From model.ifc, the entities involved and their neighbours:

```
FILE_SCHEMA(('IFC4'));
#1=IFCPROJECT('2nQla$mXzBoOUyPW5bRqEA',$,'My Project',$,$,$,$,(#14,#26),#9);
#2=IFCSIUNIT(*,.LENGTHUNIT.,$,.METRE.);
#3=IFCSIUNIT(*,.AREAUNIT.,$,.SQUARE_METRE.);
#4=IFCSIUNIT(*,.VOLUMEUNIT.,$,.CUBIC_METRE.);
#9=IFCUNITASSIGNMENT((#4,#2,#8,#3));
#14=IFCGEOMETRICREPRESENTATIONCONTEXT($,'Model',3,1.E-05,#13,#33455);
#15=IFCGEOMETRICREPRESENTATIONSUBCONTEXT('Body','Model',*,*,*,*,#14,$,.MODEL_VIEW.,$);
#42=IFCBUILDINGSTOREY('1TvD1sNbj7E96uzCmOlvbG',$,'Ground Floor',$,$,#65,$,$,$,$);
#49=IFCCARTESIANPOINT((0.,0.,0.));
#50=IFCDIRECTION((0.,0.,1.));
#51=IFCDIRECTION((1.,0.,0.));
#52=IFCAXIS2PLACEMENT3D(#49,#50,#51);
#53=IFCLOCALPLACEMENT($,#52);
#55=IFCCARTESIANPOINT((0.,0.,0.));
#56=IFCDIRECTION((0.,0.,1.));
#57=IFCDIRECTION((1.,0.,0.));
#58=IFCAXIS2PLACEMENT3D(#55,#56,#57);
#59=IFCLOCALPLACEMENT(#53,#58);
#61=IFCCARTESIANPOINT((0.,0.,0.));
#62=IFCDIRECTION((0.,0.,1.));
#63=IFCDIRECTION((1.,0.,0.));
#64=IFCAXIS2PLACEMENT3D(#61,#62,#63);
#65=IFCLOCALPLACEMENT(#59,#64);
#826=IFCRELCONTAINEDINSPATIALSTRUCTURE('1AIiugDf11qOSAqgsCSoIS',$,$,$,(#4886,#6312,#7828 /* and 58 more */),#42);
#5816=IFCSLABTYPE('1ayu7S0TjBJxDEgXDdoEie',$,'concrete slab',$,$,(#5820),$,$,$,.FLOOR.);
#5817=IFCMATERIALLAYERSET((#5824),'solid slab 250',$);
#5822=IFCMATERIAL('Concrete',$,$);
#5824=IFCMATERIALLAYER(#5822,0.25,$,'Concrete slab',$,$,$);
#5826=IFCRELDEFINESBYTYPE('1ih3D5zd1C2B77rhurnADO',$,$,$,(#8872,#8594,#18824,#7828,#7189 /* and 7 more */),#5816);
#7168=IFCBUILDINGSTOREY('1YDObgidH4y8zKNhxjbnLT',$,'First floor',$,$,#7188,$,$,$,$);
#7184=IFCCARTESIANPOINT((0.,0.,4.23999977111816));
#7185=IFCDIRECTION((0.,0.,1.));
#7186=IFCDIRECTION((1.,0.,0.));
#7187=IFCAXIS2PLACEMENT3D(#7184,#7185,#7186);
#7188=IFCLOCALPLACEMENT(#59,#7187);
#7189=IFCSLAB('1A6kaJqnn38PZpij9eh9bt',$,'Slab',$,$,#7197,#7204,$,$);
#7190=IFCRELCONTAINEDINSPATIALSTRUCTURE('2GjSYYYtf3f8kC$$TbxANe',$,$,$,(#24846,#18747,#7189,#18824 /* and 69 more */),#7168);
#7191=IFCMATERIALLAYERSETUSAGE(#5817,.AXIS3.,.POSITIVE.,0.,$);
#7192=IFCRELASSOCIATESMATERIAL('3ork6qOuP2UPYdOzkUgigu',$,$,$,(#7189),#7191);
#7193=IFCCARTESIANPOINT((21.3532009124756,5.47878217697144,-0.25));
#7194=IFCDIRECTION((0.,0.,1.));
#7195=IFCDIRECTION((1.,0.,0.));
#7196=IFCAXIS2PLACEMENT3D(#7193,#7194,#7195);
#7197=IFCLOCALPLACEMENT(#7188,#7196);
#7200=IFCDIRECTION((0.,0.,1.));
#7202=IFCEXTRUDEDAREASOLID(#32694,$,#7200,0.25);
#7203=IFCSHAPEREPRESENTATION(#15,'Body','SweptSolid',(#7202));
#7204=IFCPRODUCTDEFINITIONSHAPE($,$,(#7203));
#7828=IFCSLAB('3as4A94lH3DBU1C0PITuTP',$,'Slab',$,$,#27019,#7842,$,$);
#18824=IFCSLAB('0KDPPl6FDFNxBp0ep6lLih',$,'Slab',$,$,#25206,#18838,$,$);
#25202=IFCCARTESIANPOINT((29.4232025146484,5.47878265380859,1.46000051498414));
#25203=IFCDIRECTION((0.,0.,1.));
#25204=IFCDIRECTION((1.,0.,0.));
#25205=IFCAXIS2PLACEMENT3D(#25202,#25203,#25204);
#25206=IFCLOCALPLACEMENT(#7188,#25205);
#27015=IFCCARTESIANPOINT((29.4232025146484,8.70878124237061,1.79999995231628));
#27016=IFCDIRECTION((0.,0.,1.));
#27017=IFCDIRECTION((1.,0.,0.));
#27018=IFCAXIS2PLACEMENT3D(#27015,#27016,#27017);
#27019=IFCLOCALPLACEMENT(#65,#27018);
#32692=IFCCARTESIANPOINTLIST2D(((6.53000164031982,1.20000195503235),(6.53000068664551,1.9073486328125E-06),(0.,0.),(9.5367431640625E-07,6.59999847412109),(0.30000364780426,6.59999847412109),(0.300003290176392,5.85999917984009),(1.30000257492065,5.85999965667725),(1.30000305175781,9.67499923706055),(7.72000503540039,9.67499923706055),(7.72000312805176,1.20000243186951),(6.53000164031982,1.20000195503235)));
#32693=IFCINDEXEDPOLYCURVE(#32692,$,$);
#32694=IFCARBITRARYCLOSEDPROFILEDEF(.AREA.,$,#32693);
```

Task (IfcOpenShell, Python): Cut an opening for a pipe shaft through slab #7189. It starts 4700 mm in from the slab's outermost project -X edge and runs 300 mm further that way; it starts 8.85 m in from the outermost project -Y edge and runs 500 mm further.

```python
import numpy as np
import ifcopenshell
import ifcopenshell.api.feature
import ifcopenshell.api.geometry
import ifcopenshell.api.root
import ifcopenshell.geom
import ifcopenshell.util.placement
import ifcopenshell.util.representation
import ifcopenshell.util.shape
import ifcopenshell.util.unit

model = ifcopenshell.open("model.ifc")
unit_scale = ifcopenshell.util.unit.calculate_unit_scale(model)
settings = ifcopenshell.geom.settings()


def volume(element):
    """Net volume in cubic metres, openings subtracted."""
    shape = ifcopenshell.geom.create_shape(settings, element)
    return ifcopenshell.util.shape.get_volume(shape.geometry)


slab = model.by_id(7189)
before = volume(slab)

# Extent in the slab's own axes, in metres. The edges named are its -X and -Y sides.
slab_shape = ifcopenshell.geom.create_shape(settings, slab)
vertices = ifcopenshell.util.shape.get_vertices(slab_shape.geometry)
x_min, y_min, bottom = vertices.min(axis=0)
top = vertices[:, 2].max()

opening = ifcopenshell.api.root.create_entity(model, ifc_class="IfcOpeningElement", name="Pipe shaft opening", predefined_type="OPENING")
context = ifcopenshell.util.representation.get_context(model, "Model", "Body", "MODEL_VIEW")
width, depth = 0.3, 0.5
outline = [(0.0, 0.0), (width, 0.0), (width, depth), (0.0, depth), (0.0, 0.0)]
# Overshoot both faces by 50 mm so the cut is clean.
shape = ifcopenshell.api.geometry.add_slab_representation(
    model, context=context, depth=top - bottom + 0.1, polyline=outline
)
ifcopenshell.api.geometry.assign_representation(model, product=opening, representation=shape)

matrix = ifcopenshell.util.placement.get_local_placement(slab.ObjectPlacement)
matrix[:, 3] = matrix @ np.append(np.array([x_min + 4.7, y_min + 8.85, bottom - 0.05]) / unit_scale, 1.0)
ifcopenshell.api.geometry.edit_object_placement(model, product=opening, matrix=matrix, is_si=False)
ifcopenshell.api.feature.add_feature(model, feature=opening, element=slab)

after = volume(slab)

print(f"slab volume {before:.3f} -> {after:.3f} m3")

model.write("model_edited.ifc")
```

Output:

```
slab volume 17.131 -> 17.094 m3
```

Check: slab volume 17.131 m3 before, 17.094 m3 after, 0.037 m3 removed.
